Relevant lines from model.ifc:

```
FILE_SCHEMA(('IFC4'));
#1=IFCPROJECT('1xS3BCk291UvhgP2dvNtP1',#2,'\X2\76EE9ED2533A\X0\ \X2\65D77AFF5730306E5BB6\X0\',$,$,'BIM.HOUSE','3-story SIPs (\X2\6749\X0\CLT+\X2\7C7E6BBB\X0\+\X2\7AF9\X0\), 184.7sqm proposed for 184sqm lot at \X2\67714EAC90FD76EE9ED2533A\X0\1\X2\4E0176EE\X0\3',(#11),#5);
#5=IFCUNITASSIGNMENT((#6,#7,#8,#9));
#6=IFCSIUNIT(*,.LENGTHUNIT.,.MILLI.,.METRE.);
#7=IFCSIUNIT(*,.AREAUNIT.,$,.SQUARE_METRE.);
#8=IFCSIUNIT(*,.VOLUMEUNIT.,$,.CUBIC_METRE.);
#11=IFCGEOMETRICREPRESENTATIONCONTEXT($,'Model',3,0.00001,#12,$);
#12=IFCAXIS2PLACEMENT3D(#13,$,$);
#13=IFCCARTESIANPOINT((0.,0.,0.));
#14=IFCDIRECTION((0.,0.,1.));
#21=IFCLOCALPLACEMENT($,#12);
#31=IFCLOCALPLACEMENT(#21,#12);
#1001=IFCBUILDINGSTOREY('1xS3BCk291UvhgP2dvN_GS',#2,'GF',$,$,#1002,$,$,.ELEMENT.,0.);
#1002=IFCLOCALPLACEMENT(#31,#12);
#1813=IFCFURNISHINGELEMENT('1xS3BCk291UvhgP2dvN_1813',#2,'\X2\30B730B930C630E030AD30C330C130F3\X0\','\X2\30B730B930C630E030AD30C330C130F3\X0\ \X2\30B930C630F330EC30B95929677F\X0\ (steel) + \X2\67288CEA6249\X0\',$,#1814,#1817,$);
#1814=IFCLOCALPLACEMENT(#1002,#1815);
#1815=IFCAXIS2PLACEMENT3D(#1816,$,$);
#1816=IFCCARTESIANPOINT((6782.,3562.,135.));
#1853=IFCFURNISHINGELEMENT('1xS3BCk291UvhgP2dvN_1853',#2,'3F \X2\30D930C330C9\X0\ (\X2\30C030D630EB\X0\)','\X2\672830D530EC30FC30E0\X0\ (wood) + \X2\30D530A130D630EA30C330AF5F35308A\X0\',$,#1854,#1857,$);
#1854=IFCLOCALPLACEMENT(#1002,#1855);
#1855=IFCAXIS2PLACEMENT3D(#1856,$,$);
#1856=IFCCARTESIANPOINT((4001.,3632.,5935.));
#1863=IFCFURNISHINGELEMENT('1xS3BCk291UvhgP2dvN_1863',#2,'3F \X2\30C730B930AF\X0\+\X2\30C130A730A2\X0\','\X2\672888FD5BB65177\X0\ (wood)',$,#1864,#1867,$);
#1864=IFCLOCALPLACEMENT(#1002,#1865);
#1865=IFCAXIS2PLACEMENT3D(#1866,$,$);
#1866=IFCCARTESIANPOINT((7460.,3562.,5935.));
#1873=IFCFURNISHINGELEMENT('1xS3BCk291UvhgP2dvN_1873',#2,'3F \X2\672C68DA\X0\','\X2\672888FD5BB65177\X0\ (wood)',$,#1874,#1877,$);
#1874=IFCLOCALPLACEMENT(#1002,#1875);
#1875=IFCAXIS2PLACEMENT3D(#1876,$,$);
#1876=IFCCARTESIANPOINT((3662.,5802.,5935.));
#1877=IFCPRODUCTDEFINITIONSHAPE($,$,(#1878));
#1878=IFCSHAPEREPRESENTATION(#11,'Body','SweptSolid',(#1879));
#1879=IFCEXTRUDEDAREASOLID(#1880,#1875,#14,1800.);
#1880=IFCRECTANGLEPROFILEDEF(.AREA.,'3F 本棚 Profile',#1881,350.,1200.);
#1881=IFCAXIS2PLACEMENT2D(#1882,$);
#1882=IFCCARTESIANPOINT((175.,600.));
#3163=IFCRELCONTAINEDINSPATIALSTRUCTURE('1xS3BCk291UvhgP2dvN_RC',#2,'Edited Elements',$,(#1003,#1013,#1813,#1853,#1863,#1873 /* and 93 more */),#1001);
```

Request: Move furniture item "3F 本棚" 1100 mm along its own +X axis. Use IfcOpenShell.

```python
import ifcopenshell
import ifcopenshell.api.geometry
import ifcopenshell.util.placement
import ifcopenshell.util.unit

model = ifcopenshell.open("model.ifc")
unit_scale = ifcopenshell.util.unit.calculate_unit_scale(model)

item = model.by_id(1873)
matrix = ifcopenshell.util.placement.get_local_placement(item.ObjectPlacement)
matrix[:3, 3] += matrix[:3, 0] * 1.1 / unit_scale
ifcopenshell.api.geometry.edit_object_placement(model, product=item, matrix=matrix, is_si=False)

print(ifcopenshell.util.placement.get_local_placement(item.ObjectPlacement).round(3) + 0.0)

model.write("model_v2.ifc")
```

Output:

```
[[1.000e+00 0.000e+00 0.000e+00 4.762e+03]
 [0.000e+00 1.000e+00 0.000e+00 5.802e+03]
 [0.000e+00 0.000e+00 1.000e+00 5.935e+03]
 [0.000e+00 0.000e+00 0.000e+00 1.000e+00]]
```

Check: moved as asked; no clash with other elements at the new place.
